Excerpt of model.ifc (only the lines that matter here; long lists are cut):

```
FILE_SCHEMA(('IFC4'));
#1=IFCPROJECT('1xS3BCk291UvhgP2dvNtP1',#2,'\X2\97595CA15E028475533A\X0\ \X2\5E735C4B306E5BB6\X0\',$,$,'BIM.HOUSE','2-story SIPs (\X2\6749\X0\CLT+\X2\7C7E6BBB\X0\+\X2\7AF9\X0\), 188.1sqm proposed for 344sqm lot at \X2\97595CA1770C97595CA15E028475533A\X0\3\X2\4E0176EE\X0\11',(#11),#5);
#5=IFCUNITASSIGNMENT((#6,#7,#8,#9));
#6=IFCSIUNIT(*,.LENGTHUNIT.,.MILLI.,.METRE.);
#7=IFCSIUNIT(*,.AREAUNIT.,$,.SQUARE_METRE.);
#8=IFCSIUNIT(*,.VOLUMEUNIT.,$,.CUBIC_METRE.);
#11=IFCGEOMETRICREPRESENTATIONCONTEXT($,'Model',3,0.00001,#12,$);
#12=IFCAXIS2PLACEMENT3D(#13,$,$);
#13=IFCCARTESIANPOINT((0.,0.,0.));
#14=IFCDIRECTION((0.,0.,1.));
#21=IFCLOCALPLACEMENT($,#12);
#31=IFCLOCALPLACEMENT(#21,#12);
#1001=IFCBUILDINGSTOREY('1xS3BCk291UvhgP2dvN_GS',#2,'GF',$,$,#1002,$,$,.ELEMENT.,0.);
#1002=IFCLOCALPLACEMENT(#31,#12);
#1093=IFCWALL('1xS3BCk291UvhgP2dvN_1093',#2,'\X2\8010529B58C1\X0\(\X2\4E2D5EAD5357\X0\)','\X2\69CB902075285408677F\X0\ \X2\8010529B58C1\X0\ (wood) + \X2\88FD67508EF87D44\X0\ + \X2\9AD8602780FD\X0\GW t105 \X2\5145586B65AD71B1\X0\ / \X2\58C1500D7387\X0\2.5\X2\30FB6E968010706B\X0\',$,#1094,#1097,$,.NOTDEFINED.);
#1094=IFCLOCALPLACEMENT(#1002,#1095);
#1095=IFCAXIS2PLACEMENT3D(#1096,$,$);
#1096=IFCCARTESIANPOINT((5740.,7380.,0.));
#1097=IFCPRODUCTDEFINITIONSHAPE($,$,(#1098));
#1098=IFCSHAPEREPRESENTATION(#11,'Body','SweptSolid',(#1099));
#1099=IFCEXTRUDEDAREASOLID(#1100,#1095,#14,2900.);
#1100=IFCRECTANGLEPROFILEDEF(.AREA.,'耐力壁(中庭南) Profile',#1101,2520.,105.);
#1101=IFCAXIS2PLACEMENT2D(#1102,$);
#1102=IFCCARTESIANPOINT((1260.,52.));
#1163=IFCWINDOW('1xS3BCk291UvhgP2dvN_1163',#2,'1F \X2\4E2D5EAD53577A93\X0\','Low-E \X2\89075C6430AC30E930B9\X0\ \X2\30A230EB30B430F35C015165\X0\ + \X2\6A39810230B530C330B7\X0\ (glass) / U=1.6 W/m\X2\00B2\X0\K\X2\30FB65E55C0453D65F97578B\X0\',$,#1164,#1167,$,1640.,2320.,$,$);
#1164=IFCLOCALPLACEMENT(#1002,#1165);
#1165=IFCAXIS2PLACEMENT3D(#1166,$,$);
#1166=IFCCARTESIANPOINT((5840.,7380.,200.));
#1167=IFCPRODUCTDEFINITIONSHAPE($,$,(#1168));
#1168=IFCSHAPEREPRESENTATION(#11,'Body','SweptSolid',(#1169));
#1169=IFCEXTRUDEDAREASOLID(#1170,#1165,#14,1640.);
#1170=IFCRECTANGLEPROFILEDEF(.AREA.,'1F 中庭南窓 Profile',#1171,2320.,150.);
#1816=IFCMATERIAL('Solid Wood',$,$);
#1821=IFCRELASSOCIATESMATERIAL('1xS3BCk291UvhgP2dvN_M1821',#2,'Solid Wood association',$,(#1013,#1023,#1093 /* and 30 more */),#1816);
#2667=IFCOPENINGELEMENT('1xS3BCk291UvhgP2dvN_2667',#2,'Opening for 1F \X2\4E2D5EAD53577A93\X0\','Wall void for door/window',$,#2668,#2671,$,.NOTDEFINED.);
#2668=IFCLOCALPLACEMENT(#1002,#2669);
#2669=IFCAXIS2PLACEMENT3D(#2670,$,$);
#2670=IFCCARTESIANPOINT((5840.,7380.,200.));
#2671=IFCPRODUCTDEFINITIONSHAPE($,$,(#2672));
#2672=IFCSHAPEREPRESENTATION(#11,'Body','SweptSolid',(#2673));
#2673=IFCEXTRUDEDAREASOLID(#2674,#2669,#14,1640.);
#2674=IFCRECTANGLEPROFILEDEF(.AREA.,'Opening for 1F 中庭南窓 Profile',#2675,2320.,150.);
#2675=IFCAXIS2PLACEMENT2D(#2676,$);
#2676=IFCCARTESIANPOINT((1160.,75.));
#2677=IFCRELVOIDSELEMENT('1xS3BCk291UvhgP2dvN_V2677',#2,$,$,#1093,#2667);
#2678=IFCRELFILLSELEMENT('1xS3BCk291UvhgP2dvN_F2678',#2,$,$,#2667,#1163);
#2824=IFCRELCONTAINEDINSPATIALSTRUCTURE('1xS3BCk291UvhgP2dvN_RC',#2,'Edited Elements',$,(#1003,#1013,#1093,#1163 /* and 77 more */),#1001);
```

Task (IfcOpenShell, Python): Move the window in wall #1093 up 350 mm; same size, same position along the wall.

```python
import numpy as np
import ifcopenshell
import ifcopenshell.api.geometry
import ifcopenshell.util.placement
import ifcopenshell.util.unit

model = ifcopenshell.open("model.ifc")
unit_scale = ifcopenshell.util.unit.calculate_unit_scale(model)

window = model.by_guid("1xS3BCk291UvhgP2dvN_1163")
opening = window.FillsVoids[0].RelatingOpeningElement
dz = 0.35 / unit_scale

shift = np.array([0.0, 0.0, dz])
# The window is not placed relative to its opening, so move both.
for product in (opening, window):
    matrix = ifcopenshell.util.placement.get_local_placement(product.ObjectPlacement)
    matrix[:3, 3] += shift
    ifcopenshell.api.geometry.edit_object_placement(model, product=product, matrix=matrix, is_si=False)

print(f"moved by {dz * unit_scale:+.3f} m")

model.write("model_rev.ifc")
```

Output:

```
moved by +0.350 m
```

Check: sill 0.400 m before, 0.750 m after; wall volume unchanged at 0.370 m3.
